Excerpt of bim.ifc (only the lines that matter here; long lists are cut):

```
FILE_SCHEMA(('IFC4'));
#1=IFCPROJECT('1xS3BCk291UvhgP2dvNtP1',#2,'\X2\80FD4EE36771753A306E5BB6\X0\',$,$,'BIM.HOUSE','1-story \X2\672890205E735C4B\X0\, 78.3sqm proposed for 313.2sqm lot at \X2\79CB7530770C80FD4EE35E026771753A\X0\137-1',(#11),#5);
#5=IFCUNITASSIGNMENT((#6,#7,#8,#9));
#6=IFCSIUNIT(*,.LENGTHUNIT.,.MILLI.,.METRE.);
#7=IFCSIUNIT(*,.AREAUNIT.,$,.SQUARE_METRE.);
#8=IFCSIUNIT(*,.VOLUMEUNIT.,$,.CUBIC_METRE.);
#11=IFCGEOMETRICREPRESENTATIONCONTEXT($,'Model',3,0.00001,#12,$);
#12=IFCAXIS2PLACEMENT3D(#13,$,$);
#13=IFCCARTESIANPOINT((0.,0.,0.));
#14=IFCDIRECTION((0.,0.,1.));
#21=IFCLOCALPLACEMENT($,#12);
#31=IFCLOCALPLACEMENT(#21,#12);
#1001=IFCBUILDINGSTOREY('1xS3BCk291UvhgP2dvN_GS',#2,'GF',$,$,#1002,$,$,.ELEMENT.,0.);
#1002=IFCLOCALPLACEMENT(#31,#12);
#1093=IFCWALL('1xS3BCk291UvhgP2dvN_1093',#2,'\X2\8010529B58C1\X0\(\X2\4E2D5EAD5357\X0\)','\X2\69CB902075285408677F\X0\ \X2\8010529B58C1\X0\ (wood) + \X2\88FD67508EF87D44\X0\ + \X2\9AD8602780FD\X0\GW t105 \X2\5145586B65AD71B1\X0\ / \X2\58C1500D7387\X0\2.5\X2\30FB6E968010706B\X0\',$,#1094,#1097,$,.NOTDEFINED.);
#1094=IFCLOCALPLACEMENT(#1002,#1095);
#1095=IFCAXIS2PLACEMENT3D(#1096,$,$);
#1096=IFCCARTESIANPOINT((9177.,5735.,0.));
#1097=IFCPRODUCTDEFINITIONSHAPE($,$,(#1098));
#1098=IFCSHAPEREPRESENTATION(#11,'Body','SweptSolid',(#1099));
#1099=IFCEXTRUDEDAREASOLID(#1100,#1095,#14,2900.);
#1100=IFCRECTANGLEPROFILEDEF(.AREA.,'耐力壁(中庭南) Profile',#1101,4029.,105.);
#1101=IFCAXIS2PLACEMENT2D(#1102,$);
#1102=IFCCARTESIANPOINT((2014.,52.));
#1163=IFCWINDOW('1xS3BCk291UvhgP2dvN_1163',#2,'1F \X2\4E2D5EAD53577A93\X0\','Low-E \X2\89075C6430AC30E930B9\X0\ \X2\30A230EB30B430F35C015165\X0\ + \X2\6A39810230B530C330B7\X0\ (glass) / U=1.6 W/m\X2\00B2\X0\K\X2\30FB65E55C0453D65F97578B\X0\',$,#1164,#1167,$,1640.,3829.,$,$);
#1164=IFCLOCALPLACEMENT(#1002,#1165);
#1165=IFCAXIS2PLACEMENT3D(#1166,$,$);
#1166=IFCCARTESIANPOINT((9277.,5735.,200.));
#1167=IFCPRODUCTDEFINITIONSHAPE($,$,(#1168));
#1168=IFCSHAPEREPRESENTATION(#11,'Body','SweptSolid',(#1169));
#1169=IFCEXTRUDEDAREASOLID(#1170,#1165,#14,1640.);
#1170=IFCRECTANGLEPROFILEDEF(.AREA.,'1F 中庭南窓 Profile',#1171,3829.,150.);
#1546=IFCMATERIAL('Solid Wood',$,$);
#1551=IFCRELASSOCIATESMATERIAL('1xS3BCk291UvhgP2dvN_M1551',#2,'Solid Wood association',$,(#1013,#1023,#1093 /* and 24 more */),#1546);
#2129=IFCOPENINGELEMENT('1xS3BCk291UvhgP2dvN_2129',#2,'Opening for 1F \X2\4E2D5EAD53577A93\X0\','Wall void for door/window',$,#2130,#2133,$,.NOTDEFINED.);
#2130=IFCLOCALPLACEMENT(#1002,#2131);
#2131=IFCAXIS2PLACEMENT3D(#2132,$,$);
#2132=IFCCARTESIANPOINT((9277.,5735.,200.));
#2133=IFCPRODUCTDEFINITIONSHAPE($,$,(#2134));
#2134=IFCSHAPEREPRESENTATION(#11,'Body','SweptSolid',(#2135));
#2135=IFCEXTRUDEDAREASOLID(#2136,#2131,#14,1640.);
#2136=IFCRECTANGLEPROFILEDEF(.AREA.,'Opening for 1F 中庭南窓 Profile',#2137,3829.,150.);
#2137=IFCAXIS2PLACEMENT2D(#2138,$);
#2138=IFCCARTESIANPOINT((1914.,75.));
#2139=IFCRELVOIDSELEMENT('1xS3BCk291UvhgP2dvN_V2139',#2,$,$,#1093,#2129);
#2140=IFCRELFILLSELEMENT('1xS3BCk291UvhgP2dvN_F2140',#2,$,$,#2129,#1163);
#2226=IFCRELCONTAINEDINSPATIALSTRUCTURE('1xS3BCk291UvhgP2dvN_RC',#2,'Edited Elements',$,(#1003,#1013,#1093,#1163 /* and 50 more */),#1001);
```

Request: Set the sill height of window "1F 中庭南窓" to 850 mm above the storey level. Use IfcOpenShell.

```python
import numpy as np
import ifcopenshell
import ifcopenshell.api.geometry
import ifcopenshell.geom
import ifcopenshell.util.element
import ifcopenshell.util.placement
import ifcopenshell.util.shape
import ifcopenshell.util.unit

model = ifcopenshell.open("bim.ifc")
unit_scale = ifcopenshell.util.unit.calculate_unit_scale(model)

window = model.by_guid("1xS3BCk291UvhgP2dvN_1163")
opening = window.FillsVoids[0].RelatingOpeningElement
storey = ifcopenshell.util.element.get_container(window, ifc_class="IfcBuildingStorey")
level = ifcopenshell.util.placement.get_local_placement(storey.ObjectPlacement)[2, 3]

# The opening's origin need not be at the sill, so measure its lowest point.
shape = ifcopenshell.geom.create_shape(ifcopenshell.geom.settings(), opening)
bottom = ifcopenshell.util.shape.get_shape_bottom_elevation(shape, shape.geometry) / unit_scale
dz = level + 850.0 - bottom

shift = np.array([0.0, 0.0, dz])
# The window is not placed relative to its opening, so move both.
for product in (opening, window):
    matrix = ifcopenshell.util.placement.get_local_placement(product.ObjectPlacement)
    matrix[:3, 3] += shift
    ifcopenshell.api.geometry.edit_object_placement(model, product=product, matrix=matrix, is_si=False)

print(f"moved by {dz * unit_scale:+.3f} m")

model.write("bim_rev.ifc")
```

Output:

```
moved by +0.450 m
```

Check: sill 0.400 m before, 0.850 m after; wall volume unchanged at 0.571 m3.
